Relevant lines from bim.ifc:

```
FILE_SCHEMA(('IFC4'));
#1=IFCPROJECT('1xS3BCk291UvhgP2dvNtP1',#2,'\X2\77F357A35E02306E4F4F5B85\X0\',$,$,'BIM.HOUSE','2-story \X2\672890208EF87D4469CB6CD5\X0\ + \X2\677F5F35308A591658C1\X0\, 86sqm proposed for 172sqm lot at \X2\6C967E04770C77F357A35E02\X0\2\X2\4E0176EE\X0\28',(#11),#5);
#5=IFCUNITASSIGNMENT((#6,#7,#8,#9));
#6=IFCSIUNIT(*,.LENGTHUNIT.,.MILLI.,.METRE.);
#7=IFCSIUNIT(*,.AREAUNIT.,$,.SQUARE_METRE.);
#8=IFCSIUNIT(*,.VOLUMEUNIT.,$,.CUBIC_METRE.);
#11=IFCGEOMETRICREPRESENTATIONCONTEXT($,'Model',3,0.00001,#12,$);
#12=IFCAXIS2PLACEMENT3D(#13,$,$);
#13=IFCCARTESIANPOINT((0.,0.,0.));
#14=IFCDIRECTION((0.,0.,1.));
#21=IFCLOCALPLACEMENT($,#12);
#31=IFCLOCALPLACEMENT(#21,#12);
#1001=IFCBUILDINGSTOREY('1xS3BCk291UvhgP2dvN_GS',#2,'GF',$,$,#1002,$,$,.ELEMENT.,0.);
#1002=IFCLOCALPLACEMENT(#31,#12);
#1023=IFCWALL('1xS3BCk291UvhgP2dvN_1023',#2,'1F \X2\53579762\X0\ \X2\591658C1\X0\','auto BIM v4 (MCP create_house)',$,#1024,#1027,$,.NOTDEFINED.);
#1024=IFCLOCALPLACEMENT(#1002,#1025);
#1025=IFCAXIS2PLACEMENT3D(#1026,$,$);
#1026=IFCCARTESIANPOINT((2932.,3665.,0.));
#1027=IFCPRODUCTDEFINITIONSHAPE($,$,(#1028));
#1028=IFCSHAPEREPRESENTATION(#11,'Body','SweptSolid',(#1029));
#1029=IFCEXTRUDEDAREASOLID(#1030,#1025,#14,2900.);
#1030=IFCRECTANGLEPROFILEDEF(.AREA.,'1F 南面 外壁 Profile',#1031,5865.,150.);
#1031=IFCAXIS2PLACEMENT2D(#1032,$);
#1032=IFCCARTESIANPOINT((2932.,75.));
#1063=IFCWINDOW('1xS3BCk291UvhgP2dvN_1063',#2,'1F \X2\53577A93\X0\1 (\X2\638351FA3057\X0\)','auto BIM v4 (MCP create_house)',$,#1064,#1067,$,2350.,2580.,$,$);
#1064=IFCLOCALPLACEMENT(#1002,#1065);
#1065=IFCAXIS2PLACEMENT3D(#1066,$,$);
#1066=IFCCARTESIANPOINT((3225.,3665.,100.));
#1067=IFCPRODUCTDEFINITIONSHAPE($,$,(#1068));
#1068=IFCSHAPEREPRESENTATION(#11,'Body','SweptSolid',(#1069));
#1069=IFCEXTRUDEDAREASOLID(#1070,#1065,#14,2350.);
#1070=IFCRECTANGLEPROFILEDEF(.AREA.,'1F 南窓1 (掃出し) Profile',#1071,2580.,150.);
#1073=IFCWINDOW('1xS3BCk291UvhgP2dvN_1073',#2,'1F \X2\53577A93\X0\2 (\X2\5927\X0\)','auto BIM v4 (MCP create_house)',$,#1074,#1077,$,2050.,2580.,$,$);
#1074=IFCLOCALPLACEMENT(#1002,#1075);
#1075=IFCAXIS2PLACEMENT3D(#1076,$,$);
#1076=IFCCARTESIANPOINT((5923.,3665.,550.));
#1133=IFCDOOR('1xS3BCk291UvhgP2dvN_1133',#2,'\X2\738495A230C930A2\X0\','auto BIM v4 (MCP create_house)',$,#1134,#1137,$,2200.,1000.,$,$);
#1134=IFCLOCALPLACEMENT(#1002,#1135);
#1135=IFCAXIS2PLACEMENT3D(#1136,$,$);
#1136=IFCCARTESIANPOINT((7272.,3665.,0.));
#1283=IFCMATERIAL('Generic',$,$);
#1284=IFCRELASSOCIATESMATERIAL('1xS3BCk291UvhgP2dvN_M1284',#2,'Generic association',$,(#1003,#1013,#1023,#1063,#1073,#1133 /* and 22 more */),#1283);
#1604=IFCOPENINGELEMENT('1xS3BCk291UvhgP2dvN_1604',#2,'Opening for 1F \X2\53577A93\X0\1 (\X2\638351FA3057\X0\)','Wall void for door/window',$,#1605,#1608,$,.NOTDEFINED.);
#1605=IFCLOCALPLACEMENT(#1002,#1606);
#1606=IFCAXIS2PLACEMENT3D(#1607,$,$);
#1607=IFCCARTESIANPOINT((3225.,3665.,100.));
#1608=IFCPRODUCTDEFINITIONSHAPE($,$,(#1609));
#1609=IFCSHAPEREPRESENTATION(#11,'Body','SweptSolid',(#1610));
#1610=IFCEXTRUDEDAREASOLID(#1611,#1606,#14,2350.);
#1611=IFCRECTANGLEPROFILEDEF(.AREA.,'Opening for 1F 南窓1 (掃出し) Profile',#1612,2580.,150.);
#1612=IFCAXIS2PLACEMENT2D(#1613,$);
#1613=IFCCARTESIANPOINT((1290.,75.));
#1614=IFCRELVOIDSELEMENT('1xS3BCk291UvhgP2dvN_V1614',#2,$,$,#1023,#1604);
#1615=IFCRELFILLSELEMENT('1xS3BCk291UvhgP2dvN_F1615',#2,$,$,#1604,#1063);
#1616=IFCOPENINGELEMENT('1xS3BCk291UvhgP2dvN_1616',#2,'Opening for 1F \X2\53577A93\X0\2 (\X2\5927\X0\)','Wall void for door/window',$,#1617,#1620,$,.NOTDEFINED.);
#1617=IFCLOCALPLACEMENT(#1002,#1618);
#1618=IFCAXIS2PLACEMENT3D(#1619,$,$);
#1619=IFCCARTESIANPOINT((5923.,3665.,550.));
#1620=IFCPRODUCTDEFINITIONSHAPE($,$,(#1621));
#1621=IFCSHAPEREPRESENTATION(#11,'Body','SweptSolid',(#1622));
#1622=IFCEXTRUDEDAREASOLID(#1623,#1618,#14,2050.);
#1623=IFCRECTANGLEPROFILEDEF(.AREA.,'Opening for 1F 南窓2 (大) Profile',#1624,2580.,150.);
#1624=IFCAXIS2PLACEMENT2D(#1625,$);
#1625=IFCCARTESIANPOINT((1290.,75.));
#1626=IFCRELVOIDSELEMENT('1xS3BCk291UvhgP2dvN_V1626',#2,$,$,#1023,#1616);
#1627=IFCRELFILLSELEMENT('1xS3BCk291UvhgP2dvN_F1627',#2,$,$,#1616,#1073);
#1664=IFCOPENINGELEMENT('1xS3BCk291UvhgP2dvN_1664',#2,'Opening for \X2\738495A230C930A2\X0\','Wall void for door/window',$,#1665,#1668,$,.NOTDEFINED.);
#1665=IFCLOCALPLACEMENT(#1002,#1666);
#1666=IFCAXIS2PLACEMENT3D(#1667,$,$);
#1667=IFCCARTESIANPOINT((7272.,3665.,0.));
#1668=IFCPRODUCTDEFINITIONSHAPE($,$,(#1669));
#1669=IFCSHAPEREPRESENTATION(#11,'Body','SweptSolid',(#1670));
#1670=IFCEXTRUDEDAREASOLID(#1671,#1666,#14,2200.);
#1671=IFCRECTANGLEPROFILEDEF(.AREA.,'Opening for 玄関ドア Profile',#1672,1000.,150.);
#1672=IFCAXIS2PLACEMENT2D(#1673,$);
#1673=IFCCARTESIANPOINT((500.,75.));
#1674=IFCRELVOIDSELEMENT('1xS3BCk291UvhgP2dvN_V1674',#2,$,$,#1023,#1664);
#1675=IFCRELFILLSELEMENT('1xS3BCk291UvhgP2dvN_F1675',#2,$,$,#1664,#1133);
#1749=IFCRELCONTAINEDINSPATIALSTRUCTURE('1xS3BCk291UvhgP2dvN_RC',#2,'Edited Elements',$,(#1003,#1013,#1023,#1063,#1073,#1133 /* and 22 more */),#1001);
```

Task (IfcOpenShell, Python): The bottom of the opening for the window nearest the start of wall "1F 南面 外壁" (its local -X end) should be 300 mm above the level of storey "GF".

```python
import numpy as np
import ifcopenshell
import ifcopenshell.api.geometry
import ifcopenshell.geom
import ifcopenshell.util.element
import ifcopenshell.util.placement
import ifcopenshell.util.shape
import ifcopenshell.util.unit

model = ifcopenshell.open("bim.ifc")
unit_scale = ifcopenshell.util.unit.calculate_unit_scale(model)

window = model.by_guid("1xS3BCk291UvhgP2dvN_1063")
opening = window.FillsVoids[0].RelatingOpeningElement
storey = ifcopenshell.util.element.get_container(window, ifc_class="IfcBuildingStorey")
level = ifcopenshell.util.placement.get_local_placement(storey.ObjectPlacement)[2, 3]

# The opening's origin need not be at the sill, so measure its lowest point.
shape = ifcopenshell.geom.create_shape(ifcopenshell.geom.settings(), opening)
bottom = ifcopenshell.util.shape.get_shape_bottom_elevation(shape, shape.geometry) / unit_scale
dz = level + 0.3 / unit_scale - bottom

shift = np.array([0.0, 0.0, dz])
# The window is not placed relative to its opening, so move both.
for product in (opening, window):
    matrix = ifcopenshell.util.placement.get_local_placement(product.ObjectPlacement)
    matrix[:3, 3] += shift
    ifcopenshell.api.geometry.edit_object_placement(model, product=product, matrix=matrix, is_si=False)

print(f"moved by {dz * unit_scale:+.3f} m")

model.write("bim_updated.ifc")
```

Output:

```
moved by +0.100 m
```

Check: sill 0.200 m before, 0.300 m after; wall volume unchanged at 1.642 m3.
